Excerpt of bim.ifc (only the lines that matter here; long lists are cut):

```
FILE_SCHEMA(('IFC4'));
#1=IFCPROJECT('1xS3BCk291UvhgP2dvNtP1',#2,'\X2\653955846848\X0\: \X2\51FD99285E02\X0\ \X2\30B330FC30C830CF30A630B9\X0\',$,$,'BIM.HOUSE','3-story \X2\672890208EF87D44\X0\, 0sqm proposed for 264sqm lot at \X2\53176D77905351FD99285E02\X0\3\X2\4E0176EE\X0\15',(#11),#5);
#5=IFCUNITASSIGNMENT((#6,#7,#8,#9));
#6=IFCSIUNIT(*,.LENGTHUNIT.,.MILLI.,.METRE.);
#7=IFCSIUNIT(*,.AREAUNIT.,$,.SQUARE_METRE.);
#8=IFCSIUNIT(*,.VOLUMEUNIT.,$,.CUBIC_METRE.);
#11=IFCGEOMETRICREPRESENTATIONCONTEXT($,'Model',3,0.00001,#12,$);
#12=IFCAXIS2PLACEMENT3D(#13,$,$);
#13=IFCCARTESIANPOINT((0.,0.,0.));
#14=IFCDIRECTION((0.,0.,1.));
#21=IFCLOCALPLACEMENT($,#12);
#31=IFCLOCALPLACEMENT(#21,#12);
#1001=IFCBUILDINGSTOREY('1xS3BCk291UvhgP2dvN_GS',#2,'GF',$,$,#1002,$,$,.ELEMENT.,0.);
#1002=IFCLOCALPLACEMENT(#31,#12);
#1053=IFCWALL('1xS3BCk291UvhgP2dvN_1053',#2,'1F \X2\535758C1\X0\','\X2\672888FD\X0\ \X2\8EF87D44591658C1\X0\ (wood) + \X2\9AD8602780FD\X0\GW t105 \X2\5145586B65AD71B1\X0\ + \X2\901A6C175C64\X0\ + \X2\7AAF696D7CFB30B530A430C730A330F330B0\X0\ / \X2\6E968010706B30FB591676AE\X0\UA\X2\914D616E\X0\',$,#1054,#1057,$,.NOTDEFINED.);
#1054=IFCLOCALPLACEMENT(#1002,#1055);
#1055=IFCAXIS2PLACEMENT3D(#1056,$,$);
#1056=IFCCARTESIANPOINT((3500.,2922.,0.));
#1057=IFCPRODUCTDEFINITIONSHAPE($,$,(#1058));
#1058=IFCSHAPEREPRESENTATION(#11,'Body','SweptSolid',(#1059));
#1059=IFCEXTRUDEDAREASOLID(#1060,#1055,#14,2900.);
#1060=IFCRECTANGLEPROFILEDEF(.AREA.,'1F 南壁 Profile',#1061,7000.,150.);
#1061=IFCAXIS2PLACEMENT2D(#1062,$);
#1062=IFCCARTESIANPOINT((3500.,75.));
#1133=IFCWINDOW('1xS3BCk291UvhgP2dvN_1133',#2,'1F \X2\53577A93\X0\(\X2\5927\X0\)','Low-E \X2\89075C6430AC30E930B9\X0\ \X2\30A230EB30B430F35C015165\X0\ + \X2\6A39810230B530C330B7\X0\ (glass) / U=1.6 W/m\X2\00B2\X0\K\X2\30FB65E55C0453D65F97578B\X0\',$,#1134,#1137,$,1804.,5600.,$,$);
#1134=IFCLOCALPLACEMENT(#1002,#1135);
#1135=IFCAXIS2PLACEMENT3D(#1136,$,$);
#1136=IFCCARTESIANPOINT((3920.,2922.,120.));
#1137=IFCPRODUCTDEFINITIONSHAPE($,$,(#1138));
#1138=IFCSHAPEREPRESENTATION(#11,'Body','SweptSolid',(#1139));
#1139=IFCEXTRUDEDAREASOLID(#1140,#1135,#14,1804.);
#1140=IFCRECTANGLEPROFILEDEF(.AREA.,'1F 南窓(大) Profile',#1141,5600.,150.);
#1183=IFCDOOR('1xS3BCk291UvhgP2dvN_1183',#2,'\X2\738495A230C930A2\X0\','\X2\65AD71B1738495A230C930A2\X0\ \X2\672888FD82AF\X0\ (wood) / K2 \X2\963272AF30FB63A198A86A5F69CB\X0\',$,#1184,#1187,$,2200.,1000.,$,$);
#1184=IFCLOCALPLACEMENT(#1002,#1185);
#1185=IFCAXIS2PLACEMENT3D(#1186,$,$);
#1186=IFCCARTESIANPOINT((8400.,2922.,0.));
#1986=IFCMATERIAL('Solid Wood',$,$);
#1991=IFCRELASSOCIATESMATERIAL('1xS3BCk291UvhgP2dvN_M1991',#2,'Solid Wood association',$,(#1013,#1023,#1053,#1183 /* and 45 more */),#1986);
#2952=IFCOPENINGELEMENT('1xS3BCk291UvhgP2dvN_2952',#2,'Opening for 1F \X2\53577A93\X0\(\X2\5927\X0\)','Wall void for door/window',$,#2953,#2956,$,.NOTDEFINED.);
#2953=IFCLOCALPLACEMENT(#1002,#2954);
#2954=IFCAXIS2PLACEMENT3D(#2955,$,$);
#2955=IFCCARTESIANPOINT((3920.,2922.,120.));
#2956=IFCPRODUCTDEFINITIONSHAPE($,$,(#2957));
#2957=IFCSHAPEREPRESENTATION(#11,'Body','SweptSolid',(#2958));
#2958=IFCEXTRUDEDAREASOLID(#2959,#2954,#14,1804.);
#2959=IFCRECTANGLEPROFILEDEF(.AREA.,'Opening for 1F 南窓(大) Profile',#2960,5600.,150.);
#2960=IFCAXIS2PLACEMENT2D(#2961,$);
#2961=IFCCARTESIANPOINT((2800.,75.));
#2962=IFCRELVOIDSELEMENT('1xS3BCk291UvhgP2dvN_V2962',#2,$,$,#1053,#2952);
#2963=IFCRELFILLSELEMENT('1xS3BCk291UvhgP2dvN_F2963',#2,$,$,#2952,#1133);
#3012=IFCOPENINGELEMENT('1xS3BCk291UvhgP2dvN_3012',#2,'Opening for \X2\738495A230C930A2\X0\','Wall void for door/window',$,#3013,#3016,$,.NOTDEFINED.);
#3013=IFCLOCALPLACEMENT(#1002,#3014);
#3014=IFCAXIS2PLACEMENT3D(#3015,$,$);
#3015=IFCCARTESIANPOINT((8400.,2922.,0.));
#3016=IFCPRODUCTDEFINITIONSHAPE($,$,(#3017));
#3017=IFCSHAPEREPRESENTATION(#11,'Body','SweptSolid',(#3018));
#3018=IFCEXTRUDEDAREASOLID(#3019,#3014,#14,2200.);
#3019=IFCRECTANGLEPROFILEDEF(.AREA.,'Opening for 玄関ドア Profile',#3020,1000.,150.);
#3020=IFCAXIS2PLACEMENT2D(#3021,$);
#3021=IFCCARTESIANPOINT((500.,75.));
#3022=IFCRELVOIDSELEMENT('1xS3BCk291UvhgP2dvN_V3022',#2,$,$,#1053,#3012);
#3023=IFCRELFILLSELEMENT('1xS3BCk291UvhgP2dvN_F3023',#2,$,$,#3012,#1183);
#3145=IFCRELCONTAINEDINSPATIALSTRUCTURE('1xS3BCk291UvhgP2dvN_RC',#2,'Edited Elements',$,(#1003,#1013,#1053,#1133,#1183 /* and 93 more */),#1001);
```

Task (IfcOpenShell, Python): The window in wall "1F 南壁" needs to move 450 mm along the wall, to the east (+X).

```python
import ifcopenshell
import ifcopenshell.api.geometry
import ifcopenshell.util.placement
import ifcopenshell.util.unit

model = ifcopenshell.open("bim.ifc")
unit_scale = ifcopenshell.util.unit.calculate_unit_scale(model)

window = model.by_guid("1xS3BCk291UvhgP2dvN_1133")
opening = window.FillsVoids[0].RelatingOpeningElement
wall = opening.VoidsElements[0].RelatingBuildingElement

wall_matrix = ifcopenshell.util.placement.get_local_placement(wall.ObjectPlacement)
shift = wall_matrix[:3, 0] * 0.45 / unit_scale
before = ifcopenshell.util.placement.get_local_placement(window.ObjectPlacement)[:3, 3].copy()

# The window is not placed relative to its opening, so move both.
for product in (opening, window):
    matrix = ifcopenshell.util.placement.get_local_placement(product.ObjectPlacement)
    matrix[:3, 3] += shift
    ifcopenshell.api.geometry.edit_object_placement(model, product=product, matrix=matrix, is_si=False)

after = ifcopenshell.util.placement.get_local_placement(window.ObjectPlacement)[:3, 3]
print("window moved by", (after - before).round(3) + 0.0)

model.write("bim_rev.ifc")
```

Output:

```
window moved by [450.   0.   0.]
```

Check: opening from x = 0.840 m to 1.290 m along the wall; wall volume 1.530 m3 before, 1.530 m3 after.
